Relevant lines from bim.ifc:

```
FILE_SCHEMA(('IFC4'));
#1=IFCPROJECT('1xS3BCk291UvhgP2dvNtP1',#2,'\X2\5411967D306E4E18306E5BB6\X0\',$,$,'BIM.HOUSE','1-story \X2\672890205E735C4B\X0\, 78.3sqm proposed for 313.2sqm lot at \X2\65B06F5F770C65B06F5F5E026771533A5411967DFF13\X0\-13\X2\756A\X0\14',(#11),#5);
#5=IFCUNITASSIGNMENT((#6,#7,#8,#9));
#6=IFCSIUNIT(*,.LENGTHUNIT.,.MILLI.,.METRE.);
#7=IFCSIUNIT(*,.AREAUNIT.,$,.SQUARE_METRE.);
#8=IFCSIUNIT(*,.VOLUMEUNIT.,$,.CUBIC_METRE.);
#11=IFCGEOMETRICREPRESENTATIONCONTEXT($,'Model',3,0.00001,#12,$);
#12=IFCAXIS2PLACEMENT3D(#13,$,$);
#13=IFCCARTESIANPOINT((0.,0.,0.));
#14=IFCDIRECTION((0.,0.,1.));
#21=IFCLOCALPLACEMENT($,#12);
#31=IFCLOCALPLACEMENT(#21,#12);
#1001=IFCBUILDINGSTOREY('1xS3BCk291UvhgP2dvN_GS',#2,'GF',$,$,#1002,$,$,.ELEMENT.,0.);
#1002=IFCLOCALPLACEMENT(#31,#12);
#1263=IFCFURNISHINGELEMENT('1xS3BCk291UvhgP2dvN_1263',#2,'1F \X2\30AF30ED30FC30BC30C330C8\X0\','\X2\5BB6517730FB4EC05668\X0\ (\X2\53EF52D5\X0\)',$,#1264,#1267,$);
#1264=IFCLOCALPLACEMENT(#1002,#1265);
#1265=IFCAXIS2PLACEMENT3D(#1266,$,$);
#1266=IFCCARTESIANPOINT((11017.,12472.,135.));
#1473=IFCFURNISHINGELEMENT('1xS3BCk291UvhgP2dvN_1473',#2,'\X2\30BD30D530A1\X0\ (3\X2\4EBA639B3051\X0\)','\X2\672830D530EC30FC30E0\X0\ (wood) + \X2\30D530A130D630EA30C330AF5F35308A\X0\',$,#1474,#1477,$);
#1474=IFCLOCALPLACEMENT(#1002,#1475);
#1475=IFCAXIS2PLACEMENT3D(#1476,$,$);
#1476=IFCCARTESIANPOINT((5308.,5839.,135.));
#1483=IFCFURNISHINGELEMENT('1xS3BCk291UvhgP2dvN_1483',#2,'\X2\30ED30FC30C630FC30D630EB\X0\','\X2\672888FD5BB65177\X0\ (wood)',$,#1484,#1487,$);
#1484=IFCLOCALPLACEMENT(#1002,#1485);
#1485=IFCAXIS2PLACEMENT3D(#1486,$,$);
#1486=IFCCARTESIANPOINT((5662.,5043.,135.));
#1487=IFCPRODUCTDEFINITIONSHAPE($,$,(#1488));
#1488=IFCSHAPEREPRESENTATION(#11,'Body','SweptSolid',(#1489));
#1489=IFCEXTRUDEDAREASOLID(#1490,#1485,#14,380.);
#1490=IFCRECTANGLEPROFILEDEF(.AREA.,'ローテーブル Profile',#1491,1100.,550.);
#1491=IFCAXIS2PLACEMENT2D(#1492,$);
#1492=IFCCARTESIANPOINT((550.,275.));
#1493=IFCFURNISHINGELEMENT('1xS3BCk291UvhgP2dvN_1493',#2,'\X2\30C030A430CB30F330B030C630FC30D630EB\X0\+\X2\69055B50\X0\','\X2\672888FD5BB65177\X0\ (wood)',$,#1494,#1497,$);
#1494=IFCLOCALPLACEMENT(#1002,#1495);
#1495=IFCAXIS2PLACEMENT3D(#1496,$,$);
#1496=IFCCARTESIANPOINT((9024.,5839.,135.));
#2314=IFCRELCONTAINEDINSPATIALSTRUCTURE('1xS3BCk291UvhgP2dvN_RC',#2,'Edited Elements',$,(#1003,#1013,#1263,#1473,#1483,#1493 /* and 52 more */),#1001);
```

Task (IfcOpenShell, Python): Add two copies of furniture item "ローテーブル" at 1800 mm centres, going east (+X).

```python
import numpy as np
import ifcopenshell
import ifcopenshell.api.geometry
import ifcopenshell.api.root
import ifcopenshell.util.element
import ifcopenshell.util.placement
import ifcopenshell.util.unit

model = ifcopenshell.open("bim.ifc")
unit_scale = ifcopenshell.util.unit.calculate_unit_scale(model)


def reuse_history(source, copy):
    """copy_class also copies each property set's owner history, people and application; keep the originals."""
    for rel in copy.IsDefinedBy:
        if rel.is_a("IfcRelDefinesByProperties") and (history := rel.RelatingPropertyDefinition.OwnerHistory):
            rel.RelatingPropertyDefinition.OwnerHistory = source.OwnerHistory
            ifcopenshell.util.element.remove_deep2(model, history)


source = model.by_guid("1xS3BCk291UvhgP2dvN_1483")
base = ifcopenshell.util.placement.get_local_placement(source.ObjectPlacement)
step = np.array([1.0, 0.0, 0.0]) * 1.8 / unit_scale

for i in range(1, 3):
    copy = ifcopenshell.api.root.copy_class(model, product=source)
    copy.Representation = ifcopenshell.util.element.copy_deep(
        model, source.Representation, exclude=["IfcGeometricRepresentationContext", "IfcRepresentationMap"]
    )
    reuse_history(source, copy)
    matrix = base.copy()
    matrix[:3, 3] += i * step
    print("added at", matrix[:3, 3].round(3) + 0.0)
    ifcopenshell.api.geometry.edit_object_placement(model, product=copy, matrix=matrix, is_si=False)

model.write("bim_rev.ifc")
```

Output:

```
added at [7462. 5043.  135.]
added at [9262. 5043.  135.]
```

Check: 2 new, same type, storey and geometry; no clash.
